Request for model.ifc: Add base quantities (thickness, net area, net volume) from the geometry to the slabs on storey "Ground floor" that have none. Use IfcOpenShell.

First a look at what the model holds.

```python
import ifcopenshell
import ifcopenshell.util.element
import ifcopenshell.util.unit

model = ifcopenshell.open("model.ifc")
print(model.schema)
for unit_type in ("LENGTHUNIT", "AREAUNIT", "VOLUMEUNIT"):
    print(unit_type, ifcopenshell.util.unit.calculate_unit_scale(model, unit_type))
storey = next(s for s in model.by_type("IfcBuildingStorey") if s.Name == "Ground floor")
slabs = [e for e in ifcopenshell.util.element.get_decomposition(storey) if e.is_a("IfcSlab")]
for e in sorted(slabs, key=lambda e: e.id()):
    print(e.id(), e.is_a(), e.Name, list(ifcopenshell.util.element.get_psets(e, qtos_only=True)), sep=" | ")
```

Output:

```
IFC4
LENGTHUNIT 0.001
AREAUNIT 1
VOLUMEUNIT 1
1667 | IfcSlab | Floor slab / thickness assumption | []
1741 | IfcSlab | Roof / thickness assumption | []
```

```python
import ifcopenshell
import ifcopenshell.api.pset
import ifcopenshell.geom
import ifcopenshell.util.element
import ifcopenshell.util.shape
import ifcopenshell.util.unit

model = ifcopenshell.open("model.ifc")
unit_scale = ifcopenshell.util.unit.calculate_unit_scale(model)
area_scale = ifcopenshell.util.unit.calculate_unit_scale(model, "AREAUNIT")
volume_scale = ifcopenshell.util.unit.calculate_unit_scale(model, "VOLUMEUNIT")
settings = ifcopenshell.geom.settings()

storey = next(s for s in model.by_type("IfcBuildingStorey") if s.Name == "Ground floor")
slabs = [e for e in ifcopenshell.util.element.get_decomposition(storey) if e.is_a("IfcSlab")]

for e in sorted(slabs, key=lambda e: e.id()):
    if ifcopenshell.util.element.get_psets(e, qtos_only=True, should_inherit=False):
        continue
    # Geometry comes back in metres, in the element's own axes.
    shape = ifcopenshell.geom.create_shape(settings, e)
    values = {
        "Width": ifcopenshell.util.shape.get_z(shape.geometry) / unit_scale,
        "NetArea": ifcopenshell.util.shape.get_footprint_area(shape.geometry) / area_scale,
        "NetVolume": ifcopenshell.util.shape.get_volume(shape.geometry) / volume_scale,
    }
    qto = ifcopenshell.api.pset.add_qto(model, product=e, name="Qto_SlabBaseQuantities")
    ifcopenshell.api.pset.edit_qto(model, qto=qto, properties=values)
    print(e.id(), {k: round(v, 3) for k, v in values.items()})

model.write("model_v2.ifc")
```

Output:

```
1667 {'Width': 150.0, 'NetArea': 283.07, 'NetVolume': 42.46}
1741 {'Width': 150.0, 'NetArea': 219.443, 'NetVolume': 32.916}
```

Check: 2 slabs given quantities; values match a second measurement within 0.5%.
